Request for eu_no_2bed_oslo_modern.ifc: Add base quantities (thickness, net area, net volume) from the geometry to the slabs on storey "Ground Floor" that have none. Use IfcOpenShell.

First a look at what the model holds.

```python
import ifcopenshell
import ifcopenshell.util.element
import ifcopenshell.util.unit

model = ifcopenshell.open("eu_no_2bed_oslo_modern.ifc")
print(model.schema)
for unit_type in ("LENGTHUNIT", "AREAUNIT", "VOLUMEUNIT"):
    print(unit_type, ifcopenshell.util.unit.calculate_unit_scale(model, unit_type))
storey = next(s for s in model.by_type("IfcBuildingStorey") if s.Name == "Ground Floor")
slabs = [e for e in ifcopenshell.util.element.get_decomposition(storey) if e.is_a("IfcSlab")]
for e in sorted(slabs, key=lambda e: e.id()):
    print(e.id(), e.is_a(), e.Name, list(ifcopenshell.util.element.get_psets(e, qtos_only=True)), sep=" | ")
```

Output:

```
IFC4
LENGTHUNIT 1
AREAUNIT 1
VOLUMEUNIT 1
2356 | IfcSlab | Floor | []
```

```python
import ifcopenshell
import ifcopenshell.api.pset
import ifcopenshell.geom
import ifcopenshell.util.element
import ifcopenshell.util.shape
import ifcopenshell.util.unit

model = ifcopenshell.open("eu_no_2bed_oslo_modern.ifc")
unit_scale = ifcopenshell.util.unit.calculate_unit_scale(model)
area_scale = ifcopenshell.util.unit.calculate_unit_scale(model, "AREAUNIT")
volume_scale = ifcopenshell.util.unit.calculate_unit_scale(model, "VOLUMEUNIT")
settings = ifcopenshell.geom.settings()

storey = next(s for s in model.by_type("IfcBuildingStorey") if s.Name == "Ground Floor")
slabs = [e for e in ifcopenshell.util.element.get_decomposition(storey) if e.is_a("IfcSlab")]

for e in sorted(slabs, key=lambda e: e.id()):
    if ifcopenshell.util.element.get_psets(e, qtos_only=True, should_inherit=False):
        continue
    # Geometry comes back in metres, in the element's own axes.
    shape = ifcopenshell.geom.create_shape(settings, e)
    values = {
        "Width": ifcopenshell.util.shape.get_z(shape.geometry) / unit_scale,
        "NetArea": ifcopenshell.util.shape.get_footprint_area(shape.geometry) / area_scale,
        "NetVolume": ifcopenshell.util.shape.get_volume(shape.geometry) / volume_scale,
    }
    qto = ifcopenshell.api.pset.add_qto(model, product=e, name="Qto_SlabBaseQuantities")
    ifcopenshell.api.pset.edit_qto(model, qto=qto, properties=values)
    print(e.id(), {k: round(v, 3) for k, v in values.items()})

model.write("eu_no_2bed_oslo_modern_v2.ifc")
```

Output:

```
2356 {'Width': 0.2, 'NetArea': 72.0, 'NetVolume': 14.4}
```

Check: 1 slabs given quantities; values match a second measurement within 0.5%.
